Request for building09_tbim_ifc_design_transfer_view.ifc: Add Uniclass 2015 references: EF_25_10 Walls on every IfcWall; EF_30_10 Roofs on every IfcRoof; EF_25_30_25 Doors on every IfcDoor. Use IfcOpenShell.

First a look at what the model holds.

```python
import ifcopenshell

model = ifcopenshell.open("building09_tbim_ifc_design_transfer_view.ifc")
print(model.schema)
print("classifications:", [c.Name for c in model.by_type("IfcClassification")])
for ifc_class in ("IfcDoor", "IfcRoof", "IfcStair", "IfcWall", "IfcWindow"):
    print(ifc_class, len(model.by_type(ifc_class)))
```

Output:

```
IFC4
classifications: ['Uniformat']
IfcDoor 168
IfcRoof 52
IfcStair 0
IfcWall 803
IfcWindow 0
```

```python
import ifcopenshell
import ifcopenshell.api.classification

model = ifcopenshell.open("building09_tbim_ifc_design_transfer_view.ifc")

system = ifcopenshell.api.classification.add_classification(model, classification="Uniclass 2015")

codes = {
    "IfcWall": ("EF_25_10", "Walls"),
    "IfcRoof": ("EF_30_10", "Roofs"),
    "IfcDoor": ("EF_25_30_25", "Doors"),
}
for ifc_class, (code, name) in codes.items():
    products = model.by_type(ifc_class)
    ifcopenshell.api.classification.add_reference(
        model, products=products, classification=system, identification=code, name=name
    )
    print(code, len(products))

model.write("building09_tbim_ifc_design_transfer_view_v2.ifc")
```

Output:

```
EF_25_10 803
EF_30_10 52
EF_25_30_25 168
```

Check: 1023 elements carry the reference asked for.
